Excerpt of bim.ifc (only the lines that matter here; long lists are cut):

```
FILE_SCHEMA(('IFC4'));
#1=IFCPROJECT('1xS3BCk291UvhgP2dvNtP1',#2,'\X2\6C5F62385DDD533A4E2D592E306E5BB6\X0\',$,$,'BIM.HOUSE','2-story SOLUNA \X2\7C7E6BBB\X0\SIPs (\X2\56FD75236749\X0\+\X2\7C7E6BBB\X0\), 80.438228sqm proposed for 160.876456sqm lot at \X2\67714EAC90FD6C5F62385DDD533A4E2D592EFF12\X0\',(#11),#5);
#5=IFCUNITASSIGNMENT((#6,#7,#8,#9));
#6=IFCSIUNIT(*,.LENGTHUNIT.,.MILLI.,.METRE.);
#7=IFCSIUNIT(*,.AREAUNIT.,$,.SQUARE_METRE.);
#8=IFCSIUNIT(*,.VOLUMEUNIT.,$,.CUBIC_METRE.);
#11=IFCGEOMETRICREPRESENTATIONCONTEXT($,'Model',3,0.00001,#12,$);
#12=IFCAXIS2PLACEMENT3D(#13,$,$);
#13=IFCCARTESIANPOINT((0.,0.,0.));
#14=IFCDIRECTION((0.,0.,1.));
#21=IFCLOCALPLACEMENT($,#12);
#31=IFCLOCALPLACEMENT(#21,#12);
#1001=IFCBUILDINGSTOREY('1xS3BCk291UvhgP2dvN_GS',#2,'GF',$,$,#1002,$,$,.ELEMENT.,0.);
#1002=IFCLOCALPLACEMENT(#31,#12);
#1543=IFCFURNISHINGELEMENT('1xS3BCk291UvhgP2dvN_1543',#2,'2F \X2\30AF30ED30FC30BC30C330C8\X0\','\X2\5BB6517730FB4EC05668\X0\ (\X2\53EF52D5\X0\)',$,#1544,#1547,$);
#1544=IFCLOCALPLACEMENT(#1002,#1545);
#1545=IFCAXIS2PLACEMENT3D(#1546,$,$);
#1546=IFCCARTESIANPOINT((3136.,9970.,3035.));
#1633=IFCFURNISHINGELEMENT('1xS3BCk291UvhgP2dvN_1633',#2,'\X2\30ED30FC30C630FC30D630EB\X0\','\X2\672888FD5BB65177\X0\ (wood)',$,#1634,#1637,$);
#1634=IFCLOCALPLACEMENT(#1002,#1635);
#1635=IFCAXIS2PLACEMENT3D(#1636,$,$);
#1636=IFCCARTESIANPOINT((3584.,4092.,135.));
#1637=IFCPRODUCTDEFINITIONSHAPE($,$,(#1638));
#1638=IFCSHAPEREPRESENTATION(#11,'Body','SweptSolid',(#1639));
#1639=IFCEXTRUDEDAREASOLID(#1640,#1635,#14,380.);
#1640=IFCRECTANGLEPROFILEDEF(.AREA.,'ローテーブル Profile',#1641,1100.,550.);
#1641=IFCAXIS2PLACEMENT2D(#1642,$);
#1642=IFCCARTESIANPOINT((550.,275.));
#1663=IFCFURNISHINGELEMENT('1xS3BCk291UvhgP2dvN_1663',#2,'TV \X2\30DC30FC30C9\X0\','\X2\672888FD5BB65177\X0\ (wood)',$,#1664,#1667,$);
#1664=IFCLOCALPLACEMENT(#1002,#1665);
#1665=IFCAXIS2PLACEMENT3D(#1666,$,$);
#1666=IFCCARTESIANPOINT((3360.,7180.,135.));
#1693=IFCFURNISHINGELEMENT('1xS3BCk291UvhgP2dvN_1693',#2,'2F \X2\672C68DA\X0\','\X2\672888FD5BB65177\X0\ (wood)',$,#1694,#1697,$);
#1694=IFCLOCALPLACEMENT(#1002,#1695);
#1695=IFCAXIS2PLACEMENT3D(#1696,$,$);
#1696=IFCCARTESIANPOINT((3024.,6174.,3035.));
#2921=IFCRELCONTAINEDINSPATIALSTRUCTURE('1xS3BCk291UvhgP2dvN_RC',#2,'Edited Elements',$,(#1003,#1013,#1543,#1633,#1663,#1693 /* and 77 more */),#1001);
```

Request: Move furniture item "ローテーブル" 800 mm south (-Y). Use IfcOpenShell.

```python
import ifcopenshell
import ifcopenshell.api.geometry
import ifcopenshell.util.placement

model = ifcopenshell.open("bim.ifc")

item = model.by_guid("1xS3BCk291UvhgP2dvN_1633")
matrix = ifcopenshell.util.placement.get_local_placement(item.ObjectPlacement)
matrix[1, 3] -= 800.0
ifcopenshell.api.geometry.edit_object_placement(model, product=item, matrix=matrix, is_si=False)

print(ifcopenshell.util.placement.get_local_placement(item.ObjectPlacement).round(3) + 0.0)

model.write("bim_rev.ifc")
```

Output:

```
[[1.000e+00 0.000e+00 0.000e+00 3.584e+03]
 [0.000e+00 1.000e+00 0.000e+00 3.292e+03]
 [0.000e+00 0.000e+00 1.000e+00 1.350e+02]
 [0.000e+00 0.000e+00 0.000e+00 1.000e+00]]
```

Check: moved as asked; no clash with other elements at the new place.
